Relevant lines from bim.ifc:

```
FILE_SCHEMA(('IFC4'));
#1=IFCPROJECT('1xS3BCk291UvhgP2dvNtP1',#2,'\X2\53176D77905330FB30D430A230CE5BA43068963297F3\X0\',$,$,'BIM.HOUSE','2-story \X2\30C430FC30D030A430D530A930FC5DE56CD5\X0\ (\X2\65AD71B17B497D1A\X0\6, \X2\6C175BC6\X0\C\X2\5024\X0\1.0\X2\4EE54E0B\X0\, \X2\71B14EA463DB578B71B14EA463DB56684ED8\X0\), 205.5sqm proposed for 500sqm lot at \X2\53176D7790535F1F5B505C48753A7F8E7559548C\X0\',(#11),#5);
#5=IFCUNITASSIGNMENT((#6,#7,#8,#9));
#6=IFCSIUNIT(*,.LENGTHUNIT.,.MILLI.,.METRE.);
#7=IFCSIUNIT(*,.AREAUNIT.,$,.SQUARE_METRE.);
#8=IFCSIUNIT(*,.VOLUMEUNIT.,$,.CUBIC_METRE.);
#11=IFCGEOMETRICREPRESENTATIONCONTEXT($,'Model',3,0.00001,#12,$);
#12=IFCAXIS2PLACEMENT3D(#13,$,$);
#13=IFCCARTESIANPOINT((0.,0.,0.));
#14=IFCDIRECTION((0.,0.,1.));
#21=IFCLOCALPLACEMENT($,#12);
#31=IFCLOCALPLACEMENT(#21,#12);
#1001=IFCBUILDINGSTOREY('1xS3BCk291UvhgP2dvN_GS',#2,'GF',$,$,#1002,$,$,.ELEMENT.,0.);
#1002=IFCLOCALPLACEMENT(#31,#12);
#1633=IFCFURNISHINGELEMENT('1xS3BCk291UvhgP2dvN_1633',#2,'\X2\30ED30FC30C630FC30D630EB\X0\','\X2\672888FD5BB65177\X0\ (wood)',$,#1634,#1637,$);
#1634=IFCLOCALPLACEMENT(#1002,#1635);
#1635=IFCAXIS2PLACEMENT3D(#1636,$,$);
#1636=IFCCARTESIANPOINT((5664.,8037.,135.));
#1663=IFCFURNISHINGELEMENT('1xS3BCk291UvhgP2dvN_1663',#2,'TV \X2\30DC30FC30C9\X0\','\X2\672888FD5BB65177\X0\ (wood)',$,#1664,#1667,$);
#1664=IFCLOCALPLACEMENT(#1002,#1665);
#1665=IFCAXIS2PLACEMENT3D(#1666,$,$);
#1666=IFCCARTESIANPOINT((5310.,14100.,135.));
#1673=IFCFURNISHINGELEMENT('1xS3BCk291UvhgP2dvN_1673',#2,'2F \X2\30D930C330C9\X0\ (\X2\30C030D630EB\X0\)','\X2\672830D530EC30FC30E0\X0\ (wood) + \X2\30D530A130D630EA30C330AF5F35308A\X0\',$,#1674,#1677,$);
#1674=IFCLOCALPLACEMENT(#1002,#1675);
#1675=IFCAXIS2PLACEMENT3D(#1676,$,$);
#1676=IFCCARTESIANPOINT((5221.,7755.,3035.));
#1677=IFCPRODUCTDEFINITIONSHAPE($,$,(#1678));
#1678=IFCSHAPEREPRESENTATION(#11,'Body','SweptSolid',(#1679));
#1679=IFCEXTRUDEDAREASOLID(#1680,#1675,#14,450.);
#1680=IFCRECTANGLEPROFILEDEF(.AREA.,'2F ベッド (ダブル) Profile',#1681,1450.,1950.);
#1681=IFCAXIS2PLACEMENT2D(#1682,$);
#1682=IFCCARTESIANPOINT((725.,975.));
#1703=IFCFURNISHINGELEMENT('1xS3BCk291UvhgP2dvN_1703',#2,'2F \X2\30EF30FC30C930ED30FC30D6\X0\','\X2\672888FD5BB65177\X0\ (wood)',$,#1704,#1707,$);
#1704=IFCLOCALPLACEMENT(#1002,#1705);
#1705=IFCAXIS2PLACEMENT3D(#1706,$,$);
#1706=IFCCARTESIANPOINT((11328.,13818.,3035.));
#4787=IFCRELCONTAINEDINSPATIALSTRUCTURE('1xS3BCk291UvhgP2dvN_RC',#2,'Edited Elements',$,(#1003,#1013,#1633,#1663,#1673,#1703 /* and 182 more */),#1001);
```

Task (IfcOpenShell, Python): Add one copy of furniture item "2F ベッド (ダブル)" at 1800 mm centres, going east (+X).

```python
import numpy as np
import ifcopenshell
import ifcopenshell.api.geometry
import ifcopenshell.api.root
import ifcopenshell.util.element
import ifcopenshell.util.placement

model = ifcopenshell.open("bim.ifc")


def reuse_history(source, copy):
    """copy_class also copies each property set's owner history, people and application; keep the originals."""
    for rel in copy.IsDefinedBy:
        if rel.is_a("IfcRelDefinesByProperties") and (history := rel.RelatingPropertyDefinition.OwnerHistory):
            rel.RelatingPropertyDefinition.OwnerHistory = source.OwnerHistory
            ifcopenshell.util.element.remove_deep2(model, history)


source = model.by_guid("1xS3BCk291UvhgP2dvN_1673")
base = ifcopenshell.util.placement.get_local_placement(source.ObjectPlacement)
step = np.array([1.0, 0.0, 0.0]) * 1800.0

for i in range(1, 2):
    copy = ifcopenshell.api.root.copy_class(model, product=source)
    copy.Representation = ifcopenshell.util.element.copy_deep(
        model, source.Representation, exclude=["IfcGeometricRepresentationContext", "IfcRepresentationMap"]
    )
    reuse_history(source, copy)
    matrix = base.copy()
    matrix[:3, 3] += i * step
    print("added at", matrix[:3, 3].round(3) + 0.0)
    ifcopenshell.api.geometry.edit_object_placement(model, product=copy, matrix=matrix, is_si=False)

model.write("bim_updated.ifc")
```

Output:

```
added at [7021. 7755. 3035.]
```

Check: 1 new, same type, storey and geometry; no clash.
